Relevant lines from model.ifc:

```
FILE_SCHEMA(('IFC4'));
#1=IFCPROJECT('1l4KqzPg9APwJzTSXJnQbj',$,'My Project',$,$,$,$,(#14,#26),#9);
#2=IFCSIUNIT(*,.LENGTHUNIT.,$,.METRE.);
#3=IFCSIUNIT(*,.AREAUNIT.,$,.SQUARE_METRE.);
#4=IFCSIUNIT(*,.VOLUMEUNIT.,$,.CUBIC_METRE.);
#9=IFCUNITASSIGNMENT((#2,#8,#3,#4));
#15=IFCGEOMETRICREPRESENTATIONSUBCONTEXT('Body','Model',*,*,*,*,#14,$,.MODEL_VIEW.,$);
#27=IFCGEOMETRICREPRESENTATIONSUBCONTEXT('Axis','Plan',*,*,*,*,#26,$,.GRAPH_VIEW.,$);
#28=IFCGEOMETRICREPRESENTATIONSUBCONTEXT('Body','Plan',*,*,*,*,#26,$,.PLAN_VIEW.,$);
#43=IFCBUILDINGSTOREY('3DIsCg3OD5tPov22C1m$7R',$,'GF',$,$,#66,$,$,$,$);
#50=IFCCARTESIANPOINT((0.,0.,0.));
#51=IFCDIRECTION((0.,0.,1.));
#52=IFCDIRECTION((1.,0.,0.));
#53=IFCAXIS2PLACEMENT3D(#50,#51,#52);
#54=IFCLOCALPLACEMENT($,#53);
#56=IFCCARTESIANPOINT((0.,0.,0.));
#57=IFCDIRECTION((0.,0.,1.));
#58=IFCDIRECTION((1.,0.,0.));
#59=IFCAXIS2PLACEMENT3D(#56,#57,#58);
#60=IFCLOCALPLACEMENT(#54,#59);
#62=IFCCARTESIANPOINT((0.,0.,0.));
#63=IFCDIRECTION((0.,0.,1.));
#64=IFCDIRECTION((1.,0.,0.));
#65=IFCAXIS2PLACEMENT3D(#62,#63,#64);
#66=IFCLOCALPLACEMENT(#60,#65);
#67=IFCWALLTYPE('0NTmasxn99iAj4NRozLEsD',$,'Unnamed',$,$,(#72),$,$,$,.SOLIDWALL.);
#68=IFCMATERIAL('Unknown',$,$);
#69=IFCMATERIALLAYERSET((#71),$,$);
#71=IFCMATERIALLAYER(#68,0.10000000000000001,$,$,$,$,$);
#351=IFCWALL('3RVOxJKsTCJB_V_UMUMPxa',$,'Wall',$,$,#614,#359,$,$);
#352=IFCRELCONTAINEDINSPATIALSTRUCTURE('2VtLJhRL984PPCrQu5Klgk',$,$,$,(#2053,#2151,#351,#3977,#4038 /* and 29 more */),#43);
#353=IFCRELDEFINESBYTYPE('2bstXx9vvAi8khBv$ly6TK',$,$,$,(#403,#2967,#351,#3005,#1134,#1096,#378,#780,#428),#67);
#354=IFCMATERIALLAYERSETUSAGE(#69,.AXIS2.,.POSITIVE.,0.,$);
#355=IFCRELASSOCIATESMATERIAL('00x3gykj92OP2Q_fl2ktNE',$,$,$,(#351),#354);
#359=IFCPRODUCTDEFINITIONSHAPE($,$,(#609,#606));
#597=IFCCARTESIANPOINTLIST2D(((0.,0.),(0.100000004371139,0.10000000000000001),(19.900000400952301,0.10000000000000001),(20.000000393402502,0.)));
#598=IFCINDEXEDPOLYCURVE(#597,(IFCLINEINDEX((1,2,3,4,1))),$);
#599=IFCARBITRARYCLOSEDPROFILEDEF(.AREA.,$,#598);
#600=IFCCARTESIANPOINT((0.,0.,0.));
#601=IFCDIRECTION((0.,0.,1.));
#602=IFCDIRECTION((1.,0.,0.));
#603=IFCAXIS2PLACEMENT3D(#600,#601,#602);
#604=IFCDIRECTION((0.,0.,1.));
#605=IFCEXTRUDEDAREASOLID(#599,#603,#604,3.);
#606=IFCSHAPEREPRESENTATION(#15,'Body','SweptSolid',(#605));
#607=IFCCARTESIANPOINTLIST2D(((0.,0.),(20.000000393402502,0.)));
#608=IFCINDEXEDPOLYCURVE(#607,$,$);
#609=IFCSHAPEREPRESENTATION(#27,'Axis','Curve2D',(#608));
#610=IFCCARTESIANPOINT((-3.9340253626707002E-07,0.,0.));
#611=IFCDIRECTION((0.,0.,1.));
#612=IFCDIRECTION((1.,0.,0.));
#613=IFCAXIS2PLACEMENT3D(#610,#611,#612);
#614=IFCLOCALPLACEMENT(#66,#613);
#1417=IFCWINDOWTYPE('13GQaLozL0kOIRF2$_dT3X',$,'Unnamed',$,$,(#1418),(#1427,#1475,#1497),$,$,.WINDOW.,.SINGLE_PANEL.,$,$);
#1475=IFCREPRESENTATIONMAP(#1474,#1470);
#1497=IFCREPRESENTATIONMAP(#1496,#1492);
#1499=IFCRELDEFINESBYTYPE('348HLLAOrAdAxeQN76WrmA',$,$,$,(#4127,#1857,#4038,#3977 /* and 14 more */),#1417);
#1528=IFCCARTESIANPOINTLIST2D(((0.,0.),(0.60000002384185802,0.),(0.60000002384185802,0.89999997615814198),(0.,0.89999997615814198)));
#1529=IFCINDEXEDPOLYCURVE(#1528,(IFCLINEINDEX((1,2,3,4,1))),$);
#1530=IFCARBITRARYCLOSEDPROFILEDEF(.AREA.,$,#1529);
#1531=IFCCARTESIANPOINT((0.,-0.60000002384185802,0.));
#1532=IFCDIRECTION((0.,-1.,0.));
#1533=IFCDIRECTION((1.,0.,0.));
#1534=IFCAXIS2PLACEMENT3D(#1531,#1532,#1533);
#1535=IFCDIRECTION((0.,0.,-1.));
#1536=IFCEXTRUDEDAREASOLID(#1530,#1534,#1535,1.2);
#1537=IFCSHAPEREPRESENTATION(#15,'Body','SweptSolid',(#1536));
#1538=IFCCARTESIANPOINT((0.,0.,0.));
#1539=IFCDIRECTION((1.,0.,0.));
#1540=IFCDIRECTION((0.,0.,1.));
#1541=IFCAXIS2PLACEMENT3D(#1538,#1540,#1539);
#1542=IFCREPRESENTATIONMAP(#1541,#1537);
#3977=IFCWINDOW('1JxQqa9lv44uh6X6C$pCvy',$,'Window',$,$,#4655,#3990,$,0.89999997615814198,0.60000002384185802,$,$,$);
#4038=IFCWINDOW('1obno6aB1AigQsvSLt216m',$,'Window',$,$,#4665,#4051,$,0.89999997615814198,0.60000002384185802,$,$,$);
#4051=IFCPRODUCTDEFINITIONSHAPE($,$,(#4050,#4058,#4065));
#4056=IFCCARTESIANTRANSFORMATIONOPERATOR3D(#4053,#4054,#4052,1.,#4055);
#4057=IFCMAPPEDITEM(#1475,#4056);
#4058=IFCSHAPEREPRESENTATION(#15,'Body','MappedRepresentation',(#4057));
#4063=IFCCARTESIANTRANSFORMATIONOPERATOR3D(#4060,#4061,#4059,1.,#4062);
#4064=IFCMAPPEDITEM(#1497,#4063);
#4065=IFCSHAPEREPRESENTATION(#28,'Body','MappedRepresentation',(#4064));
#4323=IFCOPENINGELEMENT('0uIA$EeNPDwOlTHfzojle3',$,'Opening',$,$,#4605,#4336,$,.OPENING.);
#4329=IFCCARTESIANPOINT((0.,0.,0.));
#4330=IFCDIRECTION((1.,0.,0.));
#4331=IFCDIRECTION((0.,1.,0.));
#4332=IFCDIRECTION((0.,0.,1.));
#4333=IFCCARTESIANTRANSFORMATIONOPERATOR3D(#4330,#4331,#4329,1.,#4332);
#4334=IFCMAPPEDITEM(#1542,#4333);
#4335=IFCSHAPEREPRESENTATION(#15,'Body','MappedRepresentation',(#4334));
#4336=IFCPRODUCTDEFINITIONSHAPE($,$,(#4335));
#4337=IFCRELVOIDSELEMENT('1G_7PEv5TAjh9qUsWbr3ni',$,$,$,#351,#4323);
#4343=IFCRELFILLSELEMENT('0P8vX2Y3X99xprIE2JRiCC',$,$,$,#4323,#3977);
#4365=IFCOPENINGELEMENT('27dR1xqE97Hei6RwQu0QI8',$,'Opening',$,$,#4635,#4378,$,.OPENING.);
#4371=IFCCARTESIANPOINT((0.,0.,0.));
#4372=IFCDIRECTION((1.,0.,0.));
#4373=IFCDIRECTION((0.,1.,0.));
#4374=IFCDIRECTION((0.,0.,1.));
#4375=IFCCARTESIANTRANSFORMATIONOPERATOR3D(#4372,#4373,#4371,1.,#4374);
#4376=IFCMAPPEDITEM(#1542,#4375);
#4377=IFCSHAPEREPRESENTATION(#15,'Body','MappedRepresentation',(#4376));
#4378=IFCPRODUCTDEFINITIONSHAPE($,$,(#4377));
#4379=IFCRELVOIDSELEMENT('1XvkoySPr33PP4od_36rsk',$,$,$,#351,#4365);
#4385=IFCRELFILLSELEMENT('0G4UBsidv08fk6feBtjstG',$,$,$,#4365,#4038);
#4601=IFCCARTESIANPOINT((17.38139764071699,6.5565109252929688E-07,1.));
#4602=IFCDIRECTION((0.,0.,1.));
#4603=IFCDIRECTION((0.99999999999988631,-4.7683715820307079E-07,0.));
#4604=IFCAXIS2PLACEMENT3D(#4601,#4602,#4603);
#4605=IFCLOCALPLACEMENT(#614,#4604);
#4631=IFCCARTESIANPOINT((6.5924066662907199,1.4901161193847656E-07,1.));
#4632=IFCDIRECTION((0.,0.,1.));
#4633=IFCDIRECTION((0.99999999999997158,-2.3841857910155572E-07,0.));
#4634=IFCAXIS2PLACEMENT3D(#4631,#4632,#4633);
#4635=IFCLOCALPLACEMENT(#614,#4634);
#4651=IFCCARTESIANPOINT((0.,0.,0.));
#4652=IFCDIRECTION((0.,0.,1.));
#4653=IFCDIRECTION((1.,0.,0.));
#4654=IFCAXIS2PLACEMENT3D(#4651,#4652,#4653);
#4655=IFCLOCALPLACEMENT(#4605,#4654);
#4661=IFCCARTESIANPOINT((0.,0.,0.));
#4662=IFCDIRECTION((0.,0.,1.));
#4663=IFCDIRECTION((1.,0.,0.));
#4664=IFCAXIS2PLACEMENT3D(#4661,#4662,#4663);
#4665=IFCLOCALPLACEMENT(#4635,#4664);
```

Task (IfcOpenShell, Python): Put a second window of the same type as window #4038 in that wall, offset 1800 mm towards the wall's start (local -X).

```python
import ifcopenshell
import ifcopenshell.api.feature
import ifcopenshell.api.geometry
import ifcopenshell.api.root
import ifcopenshell.geom
import ifcopenshell.util.element
import ifcopenshell.util.placement
import ifcopenshell.util.shape

model = ifcopenshell.open("model.ifc")
settings = ifcopenshell.geom.settings()


def volume(element):
    """Net volume in cubic metres, openings subtracted."""
    shape = ifcopenshell.geom.create_shape(settings, element)
    return ifcopenshell.util.shape.get_volume(shape.geometry)


window = model.by_id(4038)
opening = window.FillsVoids[0].RelatingOpeningElement
wall = opening.VoidsElements[0].RelatingBuildingElement
before = volume(wall)
shift = ifcopenshell.util.placement.get_local_placement(wall.ObjectPlacement)[:3, 0] * -1.8

# copy_class copies the void relationship, type, container and properties, but no geometry.
new_opening = ifcopenshell.api.root.copy_class(model, product=opening)
new_opening.Representation = ifcopenshell.util.element.copy_deep(
    model, opening.Representation, exclude=["IfcGeometricRepresentationContext", "IfcRepresentationMap"]
)
new_window = ifcopenshell.api.root.copy_class(model, product=window)
new_window.Representation = ifcopenshell.util.element.copy_deep(
    model, window.Representation, exclude=["IfcGeometricRepresentationContext", "IfcRepresentationMap"]
)
ifcopenshell.api.feature.add_filling(model, opening=new_opening, element=new_window)

for old, new in ((opening, new_opening), (window, new_window)):
    matrix = ifcopenshell.util.placement.get_local_placement(old.ObjectPlacement)
    matrix[:3, 3] += shift
    ifcopenshell.api.geometry.edit_object_placement(model, product=new, matrix=matrix, is_si=False)

after = volume(wall)

print(f"wall volume {before:.3f} -> {after:.3f} m3")

model.write("model_updated.ifc")
```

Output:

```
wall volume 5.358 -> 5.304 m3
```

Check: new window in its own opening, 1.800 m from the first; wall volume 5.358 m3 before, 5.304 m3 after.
